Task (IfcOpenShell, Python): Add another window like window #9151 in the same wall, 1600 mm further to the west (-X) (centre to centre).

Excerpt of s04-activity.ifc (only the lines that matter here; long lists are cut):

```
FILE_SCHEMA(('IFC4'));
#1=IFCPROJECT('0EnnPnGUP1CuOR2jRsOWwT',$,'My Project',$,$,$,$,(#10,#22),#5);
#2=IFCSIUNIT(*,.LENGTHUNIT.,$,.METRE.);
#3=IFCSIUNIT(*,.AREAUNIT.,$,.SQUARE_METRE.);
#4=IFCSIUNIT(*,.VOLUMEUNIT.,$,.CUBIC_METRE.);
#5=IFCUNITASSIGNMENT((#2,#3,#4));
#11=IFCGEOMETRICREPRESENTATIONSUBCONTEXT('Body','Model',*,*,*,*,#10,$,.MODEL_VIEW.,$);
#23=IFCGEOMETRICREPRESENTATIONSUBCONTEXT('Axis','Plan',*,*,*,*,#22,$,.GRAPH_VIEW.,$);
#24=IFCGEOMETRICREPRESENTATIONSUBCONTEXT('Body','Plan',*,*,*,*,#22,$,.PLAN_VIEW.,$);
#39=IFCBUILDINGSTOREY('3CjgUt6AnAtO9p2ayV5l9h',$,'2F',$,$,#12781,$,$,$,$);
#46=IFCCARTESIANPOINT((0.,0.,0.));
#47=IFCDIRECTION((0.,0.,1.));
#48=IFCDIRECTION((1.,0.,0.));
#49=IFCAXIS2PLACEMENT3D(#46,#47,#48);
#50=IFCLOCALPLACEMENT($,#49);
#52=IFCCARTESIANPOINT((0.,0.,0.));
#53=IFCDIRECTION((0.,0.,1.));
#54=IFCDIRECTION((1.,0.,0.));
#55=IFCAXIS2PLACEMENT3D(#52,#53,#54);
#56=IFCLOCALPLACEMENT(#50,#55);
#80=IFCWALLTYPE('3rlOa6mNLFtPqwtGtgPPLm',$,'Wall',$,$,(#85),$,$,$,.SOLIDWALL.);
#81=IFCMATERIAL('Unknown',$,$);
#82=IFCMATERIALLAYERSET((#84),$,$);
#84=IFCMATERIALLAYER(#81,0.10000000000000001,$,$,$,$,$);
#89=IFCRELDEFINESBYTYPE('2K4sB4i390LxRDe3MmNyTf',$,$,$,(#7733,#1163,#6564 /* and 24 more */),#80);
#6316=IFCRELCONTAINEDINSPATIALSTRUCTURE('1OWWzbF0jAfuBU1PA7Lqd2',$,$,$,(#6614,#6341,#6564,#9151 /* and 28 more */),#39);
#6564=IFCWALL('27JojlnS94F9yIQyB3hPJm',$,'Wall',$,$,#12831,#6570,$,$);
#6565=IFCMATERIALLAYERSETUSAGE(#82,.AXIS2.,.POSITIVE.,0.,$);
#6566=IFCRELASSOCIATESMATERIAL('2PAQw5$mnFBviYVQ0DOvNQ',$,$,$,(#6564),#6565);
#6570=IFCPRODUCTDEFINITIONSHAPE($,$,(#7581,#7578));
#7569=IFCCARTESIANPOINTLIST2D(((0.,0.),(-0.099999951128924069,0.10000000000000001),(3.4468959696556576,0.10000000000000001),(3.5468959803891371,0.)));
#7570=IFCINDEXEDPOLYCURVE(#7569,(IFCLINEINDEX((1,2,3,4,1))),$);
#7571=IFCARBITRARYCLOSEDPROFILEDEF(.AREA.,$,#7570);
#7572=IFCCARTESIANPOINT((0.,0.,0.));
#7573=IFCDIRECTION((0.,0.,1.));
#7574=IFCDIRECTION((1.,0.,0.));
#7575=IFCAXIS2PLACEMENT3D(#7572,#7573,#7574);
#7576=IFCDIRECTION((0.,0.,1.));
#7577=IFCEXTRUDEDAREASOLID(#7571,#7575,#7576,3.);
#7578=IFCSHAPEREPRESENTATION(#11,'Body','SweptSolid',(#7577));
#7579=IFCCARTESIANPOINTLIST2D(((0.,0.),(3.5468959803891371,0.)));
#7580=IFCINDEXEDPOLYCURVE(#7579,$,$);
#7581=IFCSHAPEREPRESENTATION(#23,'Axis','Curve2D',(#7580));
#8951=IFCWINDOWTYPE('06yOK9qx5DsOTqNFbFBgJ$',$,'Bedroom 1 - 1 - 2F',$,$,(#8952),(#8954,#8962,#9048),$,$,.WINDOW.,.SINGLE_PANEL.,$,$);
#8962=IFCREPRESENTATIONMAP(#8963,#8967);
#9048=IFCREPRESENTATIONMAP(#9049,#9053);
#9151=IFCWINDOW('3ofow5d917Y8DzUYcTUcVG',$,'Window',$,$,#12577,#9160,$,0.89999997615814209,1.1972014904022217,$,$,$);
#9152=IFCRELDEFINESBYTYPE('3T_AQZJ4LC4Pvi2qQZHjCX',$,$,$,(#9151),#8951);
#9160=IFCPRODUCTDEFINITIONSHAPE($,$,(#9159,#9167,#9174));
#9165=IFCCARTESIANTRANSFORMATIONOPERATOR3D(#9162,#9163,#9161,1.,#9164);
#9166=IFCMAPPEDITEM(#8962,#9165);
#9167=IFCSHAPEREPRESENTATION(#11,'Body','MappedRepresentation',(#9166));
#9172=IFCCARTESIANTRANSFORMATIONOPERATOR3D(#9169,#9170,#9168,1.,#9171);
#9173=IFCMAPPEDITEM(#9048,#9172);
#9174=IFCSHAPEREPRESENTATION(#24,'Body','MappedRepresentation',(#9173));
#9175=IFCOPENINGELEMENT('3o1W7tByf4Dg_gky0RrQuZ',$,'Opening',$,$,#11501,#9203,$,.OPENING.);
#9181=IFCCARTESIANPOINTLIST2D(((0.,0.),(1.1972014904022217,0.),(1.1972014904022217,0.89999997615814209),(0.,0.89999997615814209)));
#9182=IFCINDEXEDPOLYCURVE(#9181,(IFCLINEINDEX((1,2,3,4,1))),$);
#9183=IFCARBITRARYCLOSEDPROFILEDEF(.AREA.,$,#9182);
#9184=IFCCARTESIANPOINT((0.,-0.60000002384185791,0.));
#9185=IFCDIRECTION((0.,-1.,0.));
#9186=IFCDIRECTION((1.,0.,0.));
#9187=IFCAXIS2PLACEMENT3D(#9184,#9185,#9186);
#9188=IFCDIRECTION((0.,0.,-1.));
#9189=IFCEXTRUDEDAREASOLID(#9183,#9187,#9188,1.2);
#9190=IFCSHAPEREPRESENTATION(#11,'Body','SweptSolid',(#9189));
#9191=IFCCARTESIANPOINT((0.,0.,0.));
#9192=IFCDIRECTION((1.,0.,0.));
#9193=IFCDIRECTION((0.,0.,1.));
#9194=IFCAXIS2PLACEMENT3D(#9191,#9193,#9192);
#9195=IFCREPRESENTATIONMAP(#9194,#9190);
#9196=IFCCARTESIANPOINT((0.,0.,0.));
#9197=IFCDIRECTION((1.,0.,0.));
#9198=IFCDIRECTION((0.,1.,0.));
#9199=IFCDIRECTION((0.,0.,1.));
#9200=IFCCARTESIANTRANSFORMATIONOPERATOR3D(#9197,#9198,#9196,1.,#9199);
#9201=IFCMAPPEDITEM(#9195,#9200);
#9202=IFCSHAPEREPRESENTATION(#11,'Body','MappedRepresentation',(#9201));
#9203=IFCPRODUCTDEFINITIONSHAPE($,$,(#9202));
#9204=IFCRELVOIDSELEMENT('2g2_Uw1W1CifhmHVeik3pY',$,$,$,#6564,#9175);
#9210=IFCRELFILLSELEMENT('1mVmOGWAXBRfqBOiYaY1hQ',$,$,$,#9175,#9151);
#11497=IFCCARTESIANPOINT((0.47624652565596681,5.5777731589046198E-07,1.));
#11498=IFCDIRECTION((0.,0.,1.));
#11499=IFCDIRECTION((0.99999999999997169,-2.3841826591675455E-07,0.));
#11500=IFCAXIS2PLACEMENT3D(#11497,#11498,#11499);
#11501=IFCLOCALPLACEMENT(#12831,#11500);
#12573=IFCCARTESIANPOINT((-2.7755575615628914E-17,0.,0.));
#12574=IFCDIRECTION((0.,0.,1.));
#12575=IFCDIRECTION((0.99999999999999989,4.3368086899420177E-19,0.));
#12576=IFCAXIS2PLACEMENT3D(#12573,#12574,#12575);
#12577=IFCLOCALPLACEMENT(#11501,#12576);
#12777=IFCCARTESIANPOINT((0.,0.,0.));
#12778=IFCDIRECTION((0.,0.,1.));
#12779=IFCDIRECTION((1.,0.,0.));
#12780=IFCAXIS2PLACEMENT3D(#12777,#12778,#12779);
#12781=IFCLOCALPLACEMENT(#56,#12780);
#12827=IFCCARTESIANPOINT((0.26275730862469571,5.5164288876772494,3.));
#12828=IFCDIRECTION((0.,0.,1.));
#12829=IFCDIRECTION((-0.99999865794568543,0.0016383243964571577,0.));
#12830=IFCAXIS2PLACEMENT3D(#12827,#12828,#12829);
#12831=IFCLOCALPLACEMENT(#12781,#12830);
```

```python
import ifcopenshell
import ifcopenshell.api.feature
import ifcopenshell.api.geometry
import ifcopenshell.api.root
import ifcopenshell.geom
import ifcopenshell.util.element
import ifcopenshell.util.placement
import ifcopenshell.util.shape
import ifcopenshell.util.unit

model = ifcopenshell.open("s04-activity.ifc")
unit_scale = ifcopenshell.util.unit.calculate_unit_scale(model)
settings = ifcopenshell.geom.settings()


def volume(element):
    """Net volume in cubic metres, openings subtracted."""
    shape = ifcopenshell.geom.create_shape(settings, element)
    return ifcopenshell.util.shape.get_volume(shape.geometry)


window = model.by_id(9151)
opening = window.FillsVoids[0].RelatingOpeningElement
wall = opening.VoidsElements[0].RelatingBuildingElement
before = volume(wall)
shift = ifcopenshell.util.placement.get_local_placement(wall.ObjectPlacement)[:3, 0] * 1.6 / unit_scale

# copy_class copies the void relationship, type, container and properties, but no geometry.
new_opening = ifcopenshell.api.root.copy_class(model, product=opening)
new_opening.Representation = ifcopenshell.util.element.copy_deep(
    model, opening.Representation, exclude=["IfcGeometricRepresentationContext", "IfcRepresentationMap"]
)
new_window = ifcopenshell.api.root.copy_class(model, product=window)
new_window.Representation = ifcopenshell.util.element.copy_deep(
    model, window.Representation, exclude=["IfcGeometricRepresentationContext", "IfcRepresentationMap"]
)
ifcopenshell.api.feature.add_filling(model, opening=new_opening, element=new_window)

for old, new in ((opening, new_opening), (window, new_window)):
    matrix = ifcopenshell.util.placement.get_local_placement(old.ObjectPlacement)
    matrix[:3, 3] += shift
    ifcopenshell.api.geometry.edit_object_placement(model, product=new, matrix=matrix, is_si=False)

after = volume(wall)

print(f"wall volume {before:.3f} -> {after:.3f} m3")

model.write("s04-activity-out.ifc")
```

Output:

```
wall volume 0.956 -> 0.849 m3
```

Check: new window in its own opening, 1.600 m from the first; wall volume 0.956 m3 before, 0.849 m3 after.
